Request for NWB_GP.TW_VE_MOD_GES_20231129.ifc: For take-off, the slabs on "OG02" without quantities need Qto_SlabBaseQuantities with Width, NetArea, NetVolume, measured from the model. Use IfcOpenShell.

First a look at what the model holds.

```python
import ifcopenshell
import ifcopenshell.util.element
import ifcopenshell.util.unit

model = ifcopenshell.open("NWB_GP.TW_VE_MOD_GES_20231129.ifc")
print(model.schema)
for unit_type in ("LENGTHUNIT", "AREAUNIT", "VOLUMEUNIT"):
    print(unit_type, ifcopenshell.util.unit.calculate_unit_scale(model, unit_type))
storey = next(s for s in model.by_type("IfcBuildingStorey") if s.Name == "OG02")
slabs = [e for e in ifcopenshell.util.element.get_decomposition(storey) if e.is_a("IfcSlab")]
for e in sorted(slabs, key=lambda e: e.id()):
    print(e.id(), e.is_a(), e.Name, list(ifcopenshell.util.element.get_psets(e, qtos_only=True)), sep=" | ")
```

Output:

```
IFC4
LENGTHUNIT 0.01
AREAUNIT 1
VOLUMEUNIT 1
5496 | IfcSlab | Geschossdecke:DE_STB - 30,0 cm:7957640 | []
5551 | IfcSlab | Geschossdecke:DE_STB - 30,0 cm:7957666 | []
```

```python
import ifcopenshell
import ifcopenshell.api.pset
import ifcopenshell.geom
import ifcopenshell.util.element
import ifcopenshell.util.shape
import ifcopenshell.util.unit

model = ifcopenshell.open("NWB_GP.TW_VE_MOD_GES_20231129.ifc")
unit_scale = ifcopenshell.util.unit.calculate_unit_scale(model)
area_scale = ifcopenshell.util.unit.calculate_unit_scale(model, "AREAUNIT")
volume_scale = ifcopenshell.util.unit.calculate_unit_scale(model, "VOLUMEUNIT")
settings = ifcopenshell.geom.settings()

storey = next(s for s in model.by_type("IfcBuildingStorey") if s.Name == "OG02")
slabs = [e for e in ifcopenshell.util.element.get_decomposition(storey) if e.is_a("IfcSlab")]

for e in sorted(slabs, key=lambda e: e.id()):
    if ifcopenshell.util.element.get_psets(e, qtos_only=True, should_inherit=False):
        continue
    # Geometry comes back in metres, in the element's own axes.
    shape = ifcopenshell.geom.create_shape(settings, e)
    values = {
        "Width": ifcopenshell.util.shape.get_z(shape.geometry) / unit_scale,
        "NetArea": ifcopenshell.util.shape.get_footprint_area(shape.geometry) / area_scale,
        "NetVolume": ifcopenshell.util.shape.get_volume(shape.geometry) / volume_scale,
    }
    qto = ifcopenshell.api.pset.add_qto(model, product=e, name="Qto_SlabBaseQuantities")
    ifcopenshell.api.pset.edit_qto(model, qto=qto, properties=values)
    print(e.id(), {k: round(v, 3) for k, v in values.items()})

model.write("NWB_GP.TW_VE_MOD_GES_20231129_v2.ifc")
```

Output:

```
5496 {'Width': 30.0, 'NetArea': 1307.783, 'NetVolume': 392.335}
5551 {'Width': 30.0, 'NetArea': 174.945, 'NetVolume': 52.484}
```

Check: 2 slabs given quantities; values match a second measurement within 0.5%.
